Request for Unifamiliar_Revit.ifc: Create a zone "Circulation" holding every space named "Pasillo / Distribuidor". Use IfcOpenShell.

First a look at what the model holds.

```python
import ifcopenshell

model = ifcopenshell.open("Unifamiliar_Revit.ifc")
print(model.schema)
seen = {}
for space in model.by_type("IfcSpace"):
    seen[space.LongName] = seen.get(space.LongName, 0) + 1
for name, count in sorted(seen.items(), key=str):
    print(count, "x", name)
print("zones:", [z.Name for z in model.by_type("IfcZone")][:20])
```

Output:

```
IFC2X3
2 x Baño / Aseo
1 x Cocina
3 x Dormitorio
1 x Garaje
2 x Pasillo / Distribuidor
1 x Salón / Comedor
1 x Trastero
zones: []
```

```python
import ifcopenshell
import ifcopenshell.api.group
import ifcopenshell.api.root

model = ifcopenshell.open("Unifamiliar_Revit.ifc")

names = {"Pasillo / Distribuidor"}
spaces = [s for s in model.by_type("IfcSpace") if s.LongName in names]

zone = ifcopenshell.api.root.create_entity(model, ifc_class="IfcZone", name="Circulation")
ifcopenshell.api.group.assign_group(model, products=spaces, group=zone)
print(len(spaces), "spaces in", zone.Name)

model.write("Unifamiliar_Revit_edited.ifc")
```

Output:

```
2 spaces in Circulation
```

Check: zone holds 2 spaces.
